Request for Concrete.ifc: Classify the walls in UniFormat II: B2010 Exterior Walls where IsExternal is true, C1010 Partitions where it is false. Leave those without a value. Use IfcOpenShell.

First a look at what the model holds.

```python
import ifcopenshell
import ifcopenshell.util.element

model = ifcopenshell.open("Concrete.ifc")
print(model.schema)
print("classifications:", [c.Name for c in model.by_type("IfcClassification")])
values = [ifcopenshell.util.element.get_pset(e, "Pset_WallCommon", "IsExternal") for e in model.by_type("IfcWall")]
for value in (True, False, None):
    print("IsExternal", value, values.count(value))
```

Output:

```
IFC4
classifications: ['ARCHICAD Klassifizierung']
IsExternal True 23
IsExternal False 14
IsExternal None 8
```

```python
import ifcopenshell
import ifcopenshell.api.classification
import ifcopenshell.util.element

model = ifcopenshell.open("Concrete.ifc")

system = ifcopenshell.api.classification.add_classification(model, classification="UniFormat II")

walls = model.by_type("IfcWall")
external = {e: ifcopenshell.util.element.get_pset(e, "Pset_WallCommon", "IsExternal") for e in walls}
for flag, code, name in ((True, "B2010", "Exterior Walls"), (False, "C1010", "Partitions")):
    products = [e for e in walls if external[e] is flag]
    ifcopenshell.api.classification.add_reference(
        model, products=products, classification=system, identification=code, name=name
    )
    print(code, len(products))

model.write("Concrete_updated.ifc")
```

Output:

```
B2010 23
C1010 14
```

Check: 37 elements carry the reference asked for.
